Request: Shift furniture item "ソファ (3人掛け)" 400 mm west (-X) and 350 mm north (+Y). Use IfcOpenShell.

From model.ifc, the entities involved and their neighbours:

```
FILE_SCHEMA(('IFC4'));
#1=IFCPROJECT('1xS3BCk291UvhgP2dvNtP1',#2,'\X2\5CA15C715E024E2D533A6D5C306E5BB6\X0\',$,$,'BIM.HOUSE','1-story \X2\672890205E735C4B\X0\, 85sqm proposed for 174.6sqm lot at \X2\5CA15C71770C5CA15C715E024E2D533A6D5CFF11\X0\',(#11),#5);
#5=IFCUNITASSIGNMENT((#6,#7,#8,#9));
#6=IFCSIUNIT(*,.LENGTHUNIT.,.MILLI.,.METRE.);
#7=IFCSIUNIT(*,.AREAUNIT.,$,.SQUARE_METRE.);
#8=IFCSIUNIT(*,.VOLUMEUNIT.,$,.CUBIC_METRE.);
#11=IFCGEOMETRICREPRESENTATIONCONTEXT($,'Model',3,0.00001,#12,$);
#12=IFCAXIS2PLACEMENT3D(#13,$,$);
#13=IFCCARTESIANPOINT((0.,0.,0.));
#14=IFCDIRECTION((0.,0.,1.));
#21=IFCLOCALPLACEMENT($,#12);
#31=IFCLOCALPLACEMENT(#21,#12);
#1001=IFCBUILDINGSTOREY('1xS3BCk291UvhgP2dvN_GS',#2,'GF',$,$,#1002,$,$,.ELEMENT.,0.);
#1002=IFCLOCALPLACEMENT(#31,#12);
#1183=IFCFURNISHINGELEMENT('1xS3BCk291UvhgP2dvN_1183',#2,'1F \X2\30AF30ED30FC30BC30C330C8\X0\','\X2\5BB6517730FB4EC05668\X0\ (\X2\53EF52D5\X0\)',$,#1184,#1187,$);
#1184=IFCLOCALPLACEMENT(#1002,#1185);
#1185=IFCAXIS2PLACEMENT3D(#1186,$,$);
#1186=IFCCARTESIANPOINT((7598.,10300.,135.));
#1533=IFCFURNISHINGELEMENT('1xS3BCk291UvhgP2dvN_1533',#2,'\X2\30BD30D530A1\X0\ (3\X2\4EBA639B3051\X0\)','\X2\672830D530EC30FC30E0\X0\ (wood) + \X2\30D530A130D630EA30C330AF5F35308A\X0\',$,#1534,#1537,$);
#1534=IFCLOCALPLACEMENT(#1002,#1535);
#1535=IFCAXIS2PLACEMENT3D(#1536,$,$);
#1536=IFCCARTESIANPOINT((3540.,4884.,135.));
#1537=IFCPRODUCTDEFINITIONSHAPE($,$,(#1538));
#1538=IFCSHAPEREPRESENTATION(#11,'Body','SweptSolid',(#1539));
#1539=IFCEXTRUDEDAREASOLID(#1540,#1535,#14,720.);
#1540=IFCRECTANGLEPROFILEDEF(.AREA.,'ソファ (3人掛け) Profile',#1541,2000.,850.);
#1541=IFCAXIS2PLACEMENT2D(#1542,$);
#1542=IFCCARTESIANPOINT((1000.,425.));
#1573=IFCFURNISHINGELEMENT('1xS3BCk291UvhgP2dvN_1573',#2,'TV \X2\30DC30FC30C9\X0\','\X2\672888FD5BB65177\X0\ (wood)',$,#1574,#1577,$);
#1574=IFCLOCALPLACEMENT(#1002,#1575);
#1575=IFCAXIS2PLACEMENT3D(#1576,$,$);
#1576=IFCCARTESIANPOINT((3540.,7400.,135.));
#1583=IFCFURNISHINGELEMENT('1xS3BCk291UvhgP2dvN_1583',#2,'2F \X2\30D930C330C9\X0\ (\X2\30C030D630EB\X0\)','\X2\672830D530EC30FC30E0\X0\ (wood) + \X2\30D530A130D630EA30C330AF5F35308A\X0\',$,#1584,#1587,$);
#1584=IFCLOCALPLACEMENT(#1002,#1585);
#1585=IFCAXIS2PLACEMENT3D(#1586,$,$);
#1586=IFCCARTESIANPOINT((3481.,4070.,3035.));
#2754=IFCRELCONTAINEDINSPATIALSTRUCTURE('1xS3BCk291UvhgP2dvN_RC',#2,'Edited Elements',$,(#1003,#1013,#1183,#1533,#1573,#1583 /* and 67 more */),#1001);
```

```python
import ifcopenshell
import ifcopenshell.api.geometry
import ifcopenshell.util.placement

model = ifcopenshell.open("model.ifc")

item = model.by_id(1533)
matrix = ifcopenshell.util.placement.get_local_placement(item.ObjectPlacement)
matrix[0, 3] -= 400.0
matrix[1, 3] += 350.0
ifcopenshell.api.geometry.edit_object_placement(model, product=item, matrix=matrix, is_si=False)

print(ifcopenshell.util.placement.get_local_placement(item.ObjectPlacement).round(3) + 0.0)

model.write("model_updated.ifc")
```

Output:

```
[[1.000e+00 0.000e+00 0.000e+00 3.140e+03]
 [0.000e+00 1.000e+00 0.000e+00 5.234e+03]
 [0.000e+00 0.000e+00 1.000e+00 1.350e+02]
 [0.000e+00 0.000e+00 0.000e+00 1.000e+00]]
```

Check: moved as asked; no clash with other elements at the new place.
